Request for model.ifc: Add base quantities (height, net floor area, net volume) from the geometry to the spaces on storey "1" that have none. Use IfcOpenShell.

First a look at what the model holds.

```python
import ifcopenshell
import ifcopenshell.util.element
import ifcopenshell.util.unit

model = ifcopenshell.open("model.ifc")
print(model.schema)
for unit_type in ("LENGTHUNIT", "AREAUNIT", "VOLUMEUNIT"):
    print(unit_type, ifcopenshell.util.unit.calculate_unit_scale(model, unit_type))
storey = next(s for s in model.by_type("IfcBuildingStorey") if s.Name == "1")
spaces = [e for e in ifcopenshell.util.element.get_decomposition(storey) if e.is_a("IfcSpace")]
for e in sorted(spaces, key=lambda e: e.id()):
    print(e.id(), e.is_a(), e.Name, list(ifcopenshell.util.element.get_psets(e, qtos_only=True)), sep=" | ")
```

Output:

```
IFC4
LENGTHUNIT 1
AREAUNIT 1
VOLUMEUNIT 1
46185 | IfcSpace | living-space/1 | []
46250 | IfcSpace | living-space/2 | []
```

```python
import ifcopenshell
import ifcopenshell.api.pset
import ifcopenshell.geom
import ifcopenshell.util.element
import ifcopenshell.util.shape
import ifcopenshell.util.unit

model = ifcopenshell.open("model.ifc")
unit_scale = ifcopenshell.util.unit.calculate_unit_scale(model)
area_scale = ifcopenshell.util.unit.calculate_unit_scale(model, "AREAUNIT")
volume_scale = ifcopenshell.util.unit.calculate_unit_scale(model, "VOLUMEUNIT")
settings = ifcopenshell.geom.settings()

storey = next(s for s in model.by_type("IfcBuildingStorey") if s.Name == "1")
spaces = [e for e in ifcopenshell.util.element.get_decomposition(storey) if e.is_a("IfcSpace")]

for e in sorted(spaces, key=lambda e: e.id()):
    if ifcopenshell.util.element.get_psets(e, qtos_only=True, should_inherit=False):
        continue
    # Geometry comes back in metres, in the element's own axes.
    shape = ifcopenshell.geom.create_shape(settings, e)
    values = {
        "Height": ifcopenshell.util.shape.get_z(shape.geometry) / unit_scale,
        "NetFloorArea": ifcopenshell.util.shape.get_footprint_area(shape.geometry) / area_scale,
        "NetVolume": ifcopenshell.util.shape.get_volume(shape.geometry) / volume_scale,
    }
    qto = ifcopenshell.api.pset.add_qto(model, product=e, name="Qto_SpaceBaseQuantities")
    ifcopenshell.api.pset.edit_qto(model, qto=qto, properties=values)
    print(e.id(), {k: round(v, 3) for k, v in values.items()})

model.write("model-out.ifc")
```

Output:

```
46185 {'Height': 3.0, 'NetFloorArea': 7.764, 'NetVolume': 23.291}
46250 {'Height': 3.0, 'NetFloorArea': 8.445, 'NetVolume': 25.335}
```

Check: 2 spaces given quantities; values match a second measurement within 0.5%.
